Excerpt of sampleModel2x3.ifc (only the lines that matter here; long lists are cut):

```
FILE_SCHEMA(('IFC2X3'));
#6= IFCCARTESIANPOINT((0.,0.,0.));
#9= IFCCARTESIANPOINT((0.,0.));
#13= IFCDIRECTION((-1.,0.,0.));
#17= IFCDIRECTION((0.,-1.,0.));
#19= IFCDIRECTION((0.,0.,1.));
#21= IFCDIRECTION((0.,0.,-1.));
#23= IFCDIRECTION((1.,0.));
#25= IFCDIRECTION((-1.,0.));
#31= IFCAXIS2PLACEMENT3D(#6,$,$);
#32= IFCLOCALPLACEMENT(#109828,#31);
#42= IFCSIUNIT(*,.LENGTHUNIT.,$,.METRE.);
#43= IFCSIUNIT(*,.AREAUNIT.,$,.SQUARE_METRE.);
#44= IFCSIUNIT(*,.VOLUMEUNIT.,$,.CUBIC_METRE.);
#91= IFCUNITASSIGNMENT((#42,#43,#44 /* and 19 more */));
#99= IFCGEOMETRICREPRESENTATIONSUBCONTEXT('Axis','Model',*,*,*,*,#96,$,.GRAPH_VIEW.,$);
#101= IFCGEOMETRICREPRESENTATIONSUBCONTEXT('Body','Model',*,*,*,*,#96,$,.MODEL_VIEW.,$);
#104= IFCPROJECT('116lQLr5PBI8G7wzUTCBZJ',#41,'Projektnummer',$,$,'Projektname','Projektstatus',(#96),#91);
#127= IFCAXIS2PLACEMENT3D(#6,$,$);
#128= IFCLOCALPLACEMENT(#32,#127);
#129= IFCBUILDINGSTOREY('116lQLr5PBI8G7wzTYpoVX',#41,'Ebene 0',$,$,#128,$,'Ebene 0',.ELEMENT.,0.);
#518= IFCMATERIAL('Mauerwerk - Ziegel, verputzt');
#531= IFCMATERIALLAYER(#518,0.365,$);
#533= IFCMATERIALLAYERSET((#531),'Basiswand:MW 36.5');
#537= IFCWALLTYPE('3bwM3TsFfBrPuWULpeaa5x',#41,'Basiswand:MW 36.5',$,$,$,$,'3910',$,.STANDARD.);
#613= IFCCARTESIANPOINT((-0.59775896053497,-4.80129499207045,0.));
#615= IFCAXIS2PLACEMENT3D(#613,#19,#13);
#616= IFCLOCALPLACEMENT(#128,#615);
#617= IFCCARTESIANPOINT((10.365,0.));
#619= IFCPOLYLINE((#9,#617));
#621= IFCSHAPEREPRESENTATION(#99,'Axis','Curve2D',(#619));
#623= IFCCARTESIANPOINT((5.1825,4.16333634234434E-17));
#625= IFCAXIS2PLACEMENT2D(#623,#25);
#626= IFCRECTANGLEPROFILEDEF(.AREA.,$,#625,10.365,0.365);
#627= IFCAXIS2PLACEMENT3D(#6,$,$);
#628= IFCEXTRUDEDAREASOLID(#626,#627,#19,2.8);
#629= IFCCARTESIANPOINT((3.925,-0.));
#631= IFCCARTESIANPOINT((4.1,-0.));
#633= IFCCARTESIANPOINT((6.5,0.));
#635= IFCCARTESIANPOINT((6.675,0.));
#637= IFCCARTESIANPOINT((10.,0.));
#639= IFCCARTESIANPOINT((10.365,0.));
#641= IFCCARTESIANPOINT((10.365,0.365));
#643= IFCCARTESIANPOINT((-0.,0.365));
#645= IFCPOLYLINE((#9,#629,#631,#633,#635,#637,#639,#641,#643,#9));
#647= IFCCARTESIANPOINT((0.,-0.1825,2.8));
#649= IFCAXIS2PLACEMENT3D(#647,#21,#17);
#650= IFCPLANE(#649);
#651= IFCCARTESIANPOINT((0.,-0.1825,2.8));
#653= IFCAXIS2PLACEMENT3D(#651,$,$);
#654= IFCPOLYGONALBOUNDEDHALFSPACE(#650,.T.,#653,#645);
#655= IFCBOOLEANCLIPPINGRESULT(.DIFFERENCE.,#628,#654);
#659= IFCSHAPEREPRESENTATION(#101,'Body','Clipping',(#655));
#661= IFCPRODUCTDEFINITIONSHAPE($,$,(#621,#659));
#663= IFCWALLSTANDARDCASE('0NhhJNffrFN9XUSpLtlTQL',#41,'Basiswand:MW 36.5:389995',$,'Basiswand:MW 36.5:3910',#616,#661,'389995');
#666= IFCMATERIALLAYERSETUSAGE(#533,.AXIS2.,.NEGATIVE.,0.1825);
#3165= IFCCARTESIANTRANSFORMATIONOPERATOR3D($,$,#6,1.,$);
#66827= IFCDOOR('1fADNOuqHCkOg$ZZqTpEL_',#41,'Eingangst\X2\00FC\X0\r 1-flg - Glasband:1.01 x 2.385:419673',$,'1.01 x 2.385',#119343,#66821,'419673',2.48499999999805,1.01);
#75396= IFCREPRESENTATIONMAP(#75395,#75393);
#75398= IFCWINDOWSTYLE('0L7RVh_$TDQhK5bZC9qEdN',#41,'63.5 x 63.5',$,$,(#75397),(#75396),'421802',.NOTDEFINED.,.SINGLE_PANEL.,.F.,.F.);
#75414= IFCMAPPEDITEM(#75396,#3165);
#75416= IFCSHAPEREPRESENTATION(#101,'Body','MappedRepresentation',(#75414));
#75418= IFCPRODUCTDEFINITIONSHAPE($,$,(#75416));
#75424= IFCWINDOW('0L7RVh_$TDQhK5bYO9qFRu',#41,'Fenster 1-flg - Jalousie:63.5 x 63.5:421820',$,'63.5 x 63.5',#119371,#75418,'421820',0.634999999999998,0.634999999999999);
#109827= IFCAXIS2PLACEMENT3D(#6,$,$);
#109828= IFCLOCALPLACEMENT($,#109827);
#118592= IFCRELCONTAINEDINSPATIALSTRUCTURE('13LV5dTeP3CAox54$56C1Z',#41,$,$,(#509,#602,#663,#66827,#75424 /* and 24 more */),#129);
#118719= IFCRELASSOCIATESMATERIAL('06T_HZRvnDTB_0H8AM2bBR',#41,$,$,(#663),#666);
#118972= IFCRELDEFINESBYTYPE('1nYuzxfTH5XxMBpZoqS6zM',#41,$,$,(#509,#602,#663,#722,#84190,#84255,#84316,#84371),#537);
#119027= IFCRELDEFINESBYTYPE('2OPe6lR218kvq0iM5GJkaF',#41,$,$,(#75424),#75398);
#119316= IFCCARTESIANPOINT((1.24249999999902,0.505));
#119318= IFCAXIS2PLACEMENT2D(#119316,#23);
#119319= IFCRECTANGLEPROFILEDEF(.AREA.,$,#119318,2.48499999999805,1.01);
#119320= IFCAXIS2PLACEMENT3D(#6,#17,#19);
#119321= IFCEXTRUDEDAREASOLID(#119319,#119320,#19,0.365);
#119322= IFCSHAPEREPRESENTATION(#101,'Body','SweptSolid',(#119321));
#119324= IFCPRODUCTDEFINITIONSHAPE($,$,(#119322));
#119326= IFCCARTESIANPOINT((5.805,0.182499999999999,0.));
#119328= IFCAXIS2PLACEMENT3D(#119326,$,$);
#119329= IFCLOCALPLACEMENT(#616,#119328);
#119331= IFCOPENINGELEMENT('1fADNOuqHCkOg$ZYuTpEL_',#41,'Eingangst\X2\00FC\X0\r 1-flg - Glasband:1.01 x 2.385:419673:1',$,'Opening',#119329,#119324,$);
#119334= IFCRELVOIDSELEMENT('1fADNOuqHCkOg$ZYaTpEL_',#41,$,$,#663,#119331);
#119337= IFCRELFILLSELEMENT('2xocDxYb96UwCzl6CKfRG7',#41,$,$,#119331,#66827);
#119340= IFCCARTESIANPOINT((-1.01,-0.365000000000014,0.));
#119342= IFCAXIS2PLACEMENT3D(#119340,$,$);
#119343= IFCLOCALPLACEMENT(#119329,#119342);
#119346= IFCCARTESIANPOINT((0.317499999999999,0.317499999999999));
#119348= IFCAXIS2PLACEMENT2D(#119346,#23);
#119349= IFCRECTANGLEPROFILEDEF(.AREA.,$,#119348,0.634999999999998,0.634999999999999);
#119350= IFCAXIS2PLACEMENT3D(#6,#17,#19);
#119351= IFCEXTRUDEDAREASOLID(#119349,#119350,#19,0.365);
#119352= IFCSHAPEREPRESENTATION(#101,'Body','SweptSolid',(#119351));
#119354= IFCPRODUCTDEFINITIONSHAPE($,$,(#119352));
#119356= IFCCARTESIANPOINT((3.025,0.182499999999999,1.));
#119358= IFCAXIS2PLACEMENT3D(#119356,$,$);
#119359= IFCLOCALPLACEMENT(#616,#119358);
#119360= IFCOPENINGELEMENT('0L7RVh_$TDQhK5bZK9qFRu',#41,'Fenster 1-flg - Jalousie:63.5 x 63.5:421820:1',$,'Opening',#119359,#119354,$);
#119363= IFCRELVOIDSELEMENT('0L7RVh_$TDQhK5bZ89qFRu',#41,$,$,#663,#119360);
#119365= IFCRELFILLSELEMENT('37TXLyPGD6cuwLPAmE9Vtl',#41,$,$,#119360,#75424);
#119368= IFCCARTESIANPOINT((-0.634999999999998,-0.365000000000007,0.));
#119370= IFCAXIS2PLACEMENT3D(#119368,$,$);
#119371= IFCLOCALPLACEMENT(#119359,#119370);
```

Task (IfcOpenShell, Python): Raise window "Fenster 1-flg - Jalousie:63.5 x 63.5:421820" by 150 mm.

```python
import numpy as np
import ifcopenshell
import ifcopenshell.api.geometry
import ifcopenshell.util.placement
import ifcopenshell.util.unit

model = ifcopenshell.open("sampleModel2x3.ifc")
unit_scale = ifcopenshell.util.unit.calculate_unit_scale(model)

window = model.by_guid("0L7RVh_$TDQhK5bYO9qFRu")
opening = window.FillsVoids[0].RelatingOpeningElement
dz = 0.15 / unit_scale

shift = np.array([0.0, 0.0, dz])
# The window is placed relative to its opening, so it follows when the opening moves.
matrix = ifcopenshell.util.placement.get_local_placement(opening.ObjectPlacement)
matrix[:3, 3] += shift
ifcopenshell.api.geometry.edit_object_placement(
    model, product=opening, matrix=matrix, is_si=False, should_transform_children=True
)

print(f"moved by {dz * unit_scale:+.3f} m")

model.write("sampleModel2x3_updated.ifc")
```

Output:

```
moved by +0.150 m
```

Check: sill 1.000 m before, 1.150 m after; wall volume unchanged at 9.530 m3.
